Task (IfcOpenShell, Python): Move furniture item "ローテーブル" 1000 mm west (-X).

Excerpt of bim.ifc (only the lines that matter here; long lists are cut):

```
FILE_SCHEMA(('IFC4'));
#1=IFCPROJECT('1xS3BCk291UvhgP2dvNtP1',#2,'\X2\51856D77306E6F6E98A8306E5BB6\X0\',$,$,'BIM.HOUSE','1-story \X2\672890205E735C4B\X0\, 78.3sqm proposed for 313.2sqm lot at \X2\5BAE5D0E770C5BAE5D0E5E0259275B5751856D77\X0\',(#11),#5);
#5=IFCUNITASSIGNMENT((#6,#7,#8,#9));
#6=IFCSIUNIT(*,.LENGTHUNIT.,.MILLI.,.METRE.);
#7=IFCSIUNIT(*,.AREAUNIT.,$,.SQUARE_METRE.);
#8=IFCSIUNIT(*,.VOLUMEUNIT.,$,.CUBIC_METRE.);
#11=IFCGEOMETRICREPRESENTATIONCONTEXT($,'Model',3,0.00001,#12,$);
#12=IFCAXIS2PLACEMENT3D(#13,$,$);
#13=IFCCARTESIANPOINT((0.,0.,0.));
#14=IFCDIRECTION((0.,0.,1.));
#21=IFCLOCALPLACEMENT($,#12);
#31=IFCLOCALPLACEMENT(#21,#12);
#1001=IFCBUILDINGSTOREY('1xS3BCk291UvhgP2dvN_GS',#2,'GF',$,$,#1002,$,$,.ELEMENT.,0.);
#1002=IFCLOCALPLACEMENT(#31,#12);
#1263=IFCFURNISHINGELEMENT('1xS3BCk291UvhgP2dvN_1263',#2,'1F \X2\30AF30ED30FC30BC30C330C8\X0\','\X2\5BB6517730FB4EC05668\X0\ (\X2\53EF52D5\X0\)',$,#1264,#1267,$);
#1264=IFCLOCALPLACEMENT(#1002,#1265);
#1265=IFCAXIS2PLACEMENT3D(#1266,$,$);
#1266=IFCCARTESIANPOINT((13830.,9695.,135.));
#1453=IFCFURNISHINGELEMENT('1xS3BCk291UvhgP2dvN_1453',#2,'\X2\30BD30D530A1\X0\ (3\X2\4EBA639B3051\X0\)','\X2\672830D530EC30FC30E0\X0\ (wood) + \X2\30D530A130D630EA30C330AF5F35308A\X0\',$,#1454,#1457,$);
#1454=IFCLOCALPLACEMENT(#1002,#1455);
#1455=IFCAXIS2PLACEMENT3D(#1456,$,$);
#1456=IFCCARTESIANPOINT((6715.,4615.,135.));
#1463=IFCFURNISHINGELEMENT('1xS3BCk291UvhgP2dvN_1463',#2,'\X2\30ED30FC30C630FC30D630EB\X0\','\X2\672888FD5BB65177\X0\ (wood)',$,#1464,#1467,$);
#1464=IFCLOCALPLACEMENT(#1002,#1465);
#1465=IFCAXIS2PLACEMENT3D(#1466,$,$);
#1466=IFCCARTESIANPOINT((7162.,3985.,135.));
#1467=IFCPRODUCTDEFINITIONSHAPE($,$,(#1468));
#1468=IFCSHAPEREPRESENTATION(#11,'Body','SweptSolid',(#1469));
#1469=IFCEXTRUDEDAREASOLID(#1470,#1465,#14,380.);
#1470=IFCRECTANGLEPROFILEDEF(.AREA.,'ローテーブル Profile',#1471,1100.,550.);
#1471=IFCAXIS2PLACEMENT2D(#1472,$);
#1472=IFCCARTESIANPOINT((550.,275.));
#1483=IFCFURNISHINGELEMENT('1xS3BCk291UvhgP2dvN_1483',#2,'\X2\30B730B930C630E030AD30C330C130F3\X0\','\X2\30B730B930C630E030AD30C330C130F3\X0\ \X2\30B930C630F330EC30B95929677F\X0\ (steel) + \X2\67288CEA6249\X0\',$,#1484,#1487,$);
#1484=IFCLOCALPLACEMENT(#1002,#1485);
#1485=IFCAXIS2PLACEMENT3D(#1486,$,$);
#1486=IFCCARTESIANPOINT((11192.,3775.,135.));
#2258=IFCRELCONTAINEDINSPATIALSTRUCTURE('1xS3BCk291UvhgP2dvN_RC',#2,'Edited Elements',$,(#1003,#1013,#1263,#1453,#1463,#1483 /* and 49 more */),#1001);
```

```python
import ifcopenshell
import ifcopenshell.api.geometry
import ifcopenshell.util.placement
import ifcopenshell.util.unit

model = ifcopenshell.open("bim.ifc")
unit_scale = ifcopenshell.util.unit.calculate_unit_scale(model)

item = model.by_guid("1xS3BCk291UvhgP2dvN_1463")
matrix = ifcopenshell.util.placement.get_local_placement(item.ObjectPlacement)
matrix[0, 3] -= 1 / unit_scale
ifcopenshell.api.geometry.edit_object_placement(model, product=item, matrix=matrix, is_si=False)

print(ifcopenshell.util.placement.get_local_placement(item.ObjectPlacement).round(3) + 0.0)

model.write("bim-out.ifc")
```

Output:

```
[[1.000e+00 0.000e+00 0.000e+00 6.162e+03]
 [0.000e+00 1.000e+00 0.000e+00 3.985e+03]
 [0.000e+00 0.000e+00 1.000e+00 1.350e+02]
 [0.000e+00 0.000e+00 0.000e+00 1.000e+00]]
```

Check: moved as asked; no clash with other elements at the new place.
